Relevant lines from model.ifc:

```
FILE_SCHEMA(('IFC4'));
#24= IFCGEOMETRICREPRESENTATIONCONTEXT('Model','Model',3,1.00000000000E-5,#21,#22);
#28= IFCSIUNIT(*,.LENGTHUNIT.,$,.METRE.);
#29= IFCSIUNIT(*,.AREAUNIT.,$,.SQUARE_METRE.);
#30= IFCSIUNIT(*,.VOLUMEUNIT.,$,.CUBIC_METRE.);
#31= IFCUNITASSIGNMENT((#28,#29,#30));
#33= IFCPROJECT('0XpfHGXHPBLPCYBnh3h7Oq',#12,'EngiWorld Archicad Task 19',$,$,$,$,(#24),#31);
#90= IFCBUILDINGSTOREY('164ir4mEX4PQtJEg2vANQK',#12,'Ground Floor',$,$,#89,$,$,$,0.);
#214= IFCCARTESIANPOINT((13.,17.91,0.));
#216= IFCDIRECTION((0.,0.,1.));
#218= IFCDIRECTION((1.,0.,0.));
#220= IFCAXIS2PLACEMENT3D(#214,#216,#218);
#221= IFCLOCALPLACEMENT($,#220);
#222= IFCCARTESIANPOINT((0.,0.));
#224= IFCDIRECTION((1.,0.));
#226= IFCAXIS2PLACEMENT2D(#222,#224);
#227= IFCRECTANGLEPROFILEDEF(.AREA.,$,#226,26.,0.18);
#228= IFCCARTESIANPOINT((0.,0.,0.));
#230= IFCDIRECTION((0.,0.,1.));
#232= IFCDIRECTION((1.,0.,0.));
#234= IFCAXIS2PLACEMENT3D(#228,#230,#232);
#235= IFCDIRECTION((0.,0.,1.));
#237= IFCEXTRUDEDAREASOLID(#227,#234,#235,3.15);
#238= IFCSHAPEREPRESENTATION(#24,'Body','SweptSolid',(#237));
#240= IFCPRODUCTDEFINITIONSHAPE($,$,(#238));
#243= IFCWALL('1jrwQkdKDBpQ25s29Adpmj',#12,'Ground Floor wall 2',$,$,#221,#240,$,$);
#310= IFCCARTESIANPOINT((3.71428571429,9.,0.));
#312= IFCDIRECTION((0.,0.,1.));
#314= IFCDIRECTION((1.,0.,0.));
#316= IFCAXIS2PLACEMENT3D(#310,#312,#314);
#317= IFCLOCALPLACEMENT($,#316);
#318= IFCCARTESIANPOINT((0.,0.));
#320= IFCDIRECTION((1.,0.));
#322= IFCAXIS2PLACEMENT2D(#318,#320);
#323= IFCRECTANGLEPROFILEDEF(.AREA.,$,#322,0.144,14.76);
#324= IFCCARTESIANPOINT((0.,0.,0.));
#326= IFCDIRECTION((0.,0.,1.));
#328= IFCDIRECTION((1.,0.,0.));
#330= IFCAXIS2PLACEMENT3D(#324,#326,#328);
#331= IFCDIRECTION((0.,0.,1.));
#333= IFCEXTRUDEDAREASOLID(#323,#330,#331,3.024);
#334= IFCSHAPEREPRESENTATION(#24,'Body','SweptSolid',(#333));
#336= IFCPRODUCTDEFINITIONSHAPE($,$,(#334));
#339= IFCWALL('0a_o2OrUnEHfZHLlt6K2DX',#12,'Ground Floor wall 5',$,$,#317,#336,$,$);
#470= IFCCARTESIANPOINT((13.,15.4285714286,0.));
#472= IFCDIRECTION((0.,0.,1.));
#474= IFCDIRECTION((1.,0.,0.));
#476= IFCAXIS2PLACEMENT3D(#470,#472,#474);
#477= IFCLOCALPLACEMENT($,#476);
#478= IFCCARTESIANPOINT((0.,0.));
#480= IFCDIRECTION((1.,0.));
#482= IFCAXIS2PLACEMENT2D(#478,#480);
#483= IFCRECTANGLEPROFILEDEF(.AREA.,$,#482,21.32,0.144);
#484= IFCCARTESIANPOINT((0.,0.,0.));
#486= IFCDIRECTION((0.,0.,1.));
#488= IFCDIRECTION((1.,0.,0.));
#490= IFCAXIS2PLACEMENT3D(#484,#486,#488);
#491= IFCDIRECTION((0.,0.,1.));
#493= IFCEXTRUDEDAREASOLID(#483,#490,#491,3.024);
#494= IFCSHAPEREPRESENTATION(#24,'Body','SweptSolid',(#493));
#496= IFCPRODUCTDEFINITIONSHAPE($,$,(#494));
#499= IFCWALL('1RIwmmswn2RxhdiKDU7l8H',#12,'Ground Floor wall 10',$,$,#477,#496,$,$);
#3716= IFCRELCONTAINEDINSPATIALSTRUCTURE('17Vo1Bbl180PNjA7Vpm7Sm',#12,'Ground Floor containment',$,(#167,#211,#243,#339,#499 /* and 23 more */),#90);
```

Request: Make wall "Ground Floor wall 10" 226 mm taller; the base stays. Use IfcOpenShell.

```python
import ifcopenshell
import ifcopenshell.geom
import ifcopenshell.util.shape
import ifcopenshell.util.unit

model = ifcopenshell.open("model.ifc")
unit_scale = ifcopenshell.util.unit.calculate_unit_scale(model)
settings = ifcopenshell.geom.settings()


def volume(element):
    """Net volume in cubic metres, openings subtracted."""
    shape = ifcopenshell.geom.create_shape(settings, element)
    return ifcopenshell.util.shape.get_volume(shape.geometry)


wall = model.by_guid("1RIwmmswn2RxhdiKDU7l8H")
before = volume(wall)

body = next(r for r in wall.Representation.Representations if r.RepresentationIdentifier == "Body")
solid = body.Items[0]
old_height = solid.Depth
solid.Depth += 0.226 / unit_scale
after = volume(wall)

print(f"height {old_height:g} -> {solid.Depth:g}, volume {before:.3f} -> {after:.3f} m3")

model.write("model-out.ifc")
```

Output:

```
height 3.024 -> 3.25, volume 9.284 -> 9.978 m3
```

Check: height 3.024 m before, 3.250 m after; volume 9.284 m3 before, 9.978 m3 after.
